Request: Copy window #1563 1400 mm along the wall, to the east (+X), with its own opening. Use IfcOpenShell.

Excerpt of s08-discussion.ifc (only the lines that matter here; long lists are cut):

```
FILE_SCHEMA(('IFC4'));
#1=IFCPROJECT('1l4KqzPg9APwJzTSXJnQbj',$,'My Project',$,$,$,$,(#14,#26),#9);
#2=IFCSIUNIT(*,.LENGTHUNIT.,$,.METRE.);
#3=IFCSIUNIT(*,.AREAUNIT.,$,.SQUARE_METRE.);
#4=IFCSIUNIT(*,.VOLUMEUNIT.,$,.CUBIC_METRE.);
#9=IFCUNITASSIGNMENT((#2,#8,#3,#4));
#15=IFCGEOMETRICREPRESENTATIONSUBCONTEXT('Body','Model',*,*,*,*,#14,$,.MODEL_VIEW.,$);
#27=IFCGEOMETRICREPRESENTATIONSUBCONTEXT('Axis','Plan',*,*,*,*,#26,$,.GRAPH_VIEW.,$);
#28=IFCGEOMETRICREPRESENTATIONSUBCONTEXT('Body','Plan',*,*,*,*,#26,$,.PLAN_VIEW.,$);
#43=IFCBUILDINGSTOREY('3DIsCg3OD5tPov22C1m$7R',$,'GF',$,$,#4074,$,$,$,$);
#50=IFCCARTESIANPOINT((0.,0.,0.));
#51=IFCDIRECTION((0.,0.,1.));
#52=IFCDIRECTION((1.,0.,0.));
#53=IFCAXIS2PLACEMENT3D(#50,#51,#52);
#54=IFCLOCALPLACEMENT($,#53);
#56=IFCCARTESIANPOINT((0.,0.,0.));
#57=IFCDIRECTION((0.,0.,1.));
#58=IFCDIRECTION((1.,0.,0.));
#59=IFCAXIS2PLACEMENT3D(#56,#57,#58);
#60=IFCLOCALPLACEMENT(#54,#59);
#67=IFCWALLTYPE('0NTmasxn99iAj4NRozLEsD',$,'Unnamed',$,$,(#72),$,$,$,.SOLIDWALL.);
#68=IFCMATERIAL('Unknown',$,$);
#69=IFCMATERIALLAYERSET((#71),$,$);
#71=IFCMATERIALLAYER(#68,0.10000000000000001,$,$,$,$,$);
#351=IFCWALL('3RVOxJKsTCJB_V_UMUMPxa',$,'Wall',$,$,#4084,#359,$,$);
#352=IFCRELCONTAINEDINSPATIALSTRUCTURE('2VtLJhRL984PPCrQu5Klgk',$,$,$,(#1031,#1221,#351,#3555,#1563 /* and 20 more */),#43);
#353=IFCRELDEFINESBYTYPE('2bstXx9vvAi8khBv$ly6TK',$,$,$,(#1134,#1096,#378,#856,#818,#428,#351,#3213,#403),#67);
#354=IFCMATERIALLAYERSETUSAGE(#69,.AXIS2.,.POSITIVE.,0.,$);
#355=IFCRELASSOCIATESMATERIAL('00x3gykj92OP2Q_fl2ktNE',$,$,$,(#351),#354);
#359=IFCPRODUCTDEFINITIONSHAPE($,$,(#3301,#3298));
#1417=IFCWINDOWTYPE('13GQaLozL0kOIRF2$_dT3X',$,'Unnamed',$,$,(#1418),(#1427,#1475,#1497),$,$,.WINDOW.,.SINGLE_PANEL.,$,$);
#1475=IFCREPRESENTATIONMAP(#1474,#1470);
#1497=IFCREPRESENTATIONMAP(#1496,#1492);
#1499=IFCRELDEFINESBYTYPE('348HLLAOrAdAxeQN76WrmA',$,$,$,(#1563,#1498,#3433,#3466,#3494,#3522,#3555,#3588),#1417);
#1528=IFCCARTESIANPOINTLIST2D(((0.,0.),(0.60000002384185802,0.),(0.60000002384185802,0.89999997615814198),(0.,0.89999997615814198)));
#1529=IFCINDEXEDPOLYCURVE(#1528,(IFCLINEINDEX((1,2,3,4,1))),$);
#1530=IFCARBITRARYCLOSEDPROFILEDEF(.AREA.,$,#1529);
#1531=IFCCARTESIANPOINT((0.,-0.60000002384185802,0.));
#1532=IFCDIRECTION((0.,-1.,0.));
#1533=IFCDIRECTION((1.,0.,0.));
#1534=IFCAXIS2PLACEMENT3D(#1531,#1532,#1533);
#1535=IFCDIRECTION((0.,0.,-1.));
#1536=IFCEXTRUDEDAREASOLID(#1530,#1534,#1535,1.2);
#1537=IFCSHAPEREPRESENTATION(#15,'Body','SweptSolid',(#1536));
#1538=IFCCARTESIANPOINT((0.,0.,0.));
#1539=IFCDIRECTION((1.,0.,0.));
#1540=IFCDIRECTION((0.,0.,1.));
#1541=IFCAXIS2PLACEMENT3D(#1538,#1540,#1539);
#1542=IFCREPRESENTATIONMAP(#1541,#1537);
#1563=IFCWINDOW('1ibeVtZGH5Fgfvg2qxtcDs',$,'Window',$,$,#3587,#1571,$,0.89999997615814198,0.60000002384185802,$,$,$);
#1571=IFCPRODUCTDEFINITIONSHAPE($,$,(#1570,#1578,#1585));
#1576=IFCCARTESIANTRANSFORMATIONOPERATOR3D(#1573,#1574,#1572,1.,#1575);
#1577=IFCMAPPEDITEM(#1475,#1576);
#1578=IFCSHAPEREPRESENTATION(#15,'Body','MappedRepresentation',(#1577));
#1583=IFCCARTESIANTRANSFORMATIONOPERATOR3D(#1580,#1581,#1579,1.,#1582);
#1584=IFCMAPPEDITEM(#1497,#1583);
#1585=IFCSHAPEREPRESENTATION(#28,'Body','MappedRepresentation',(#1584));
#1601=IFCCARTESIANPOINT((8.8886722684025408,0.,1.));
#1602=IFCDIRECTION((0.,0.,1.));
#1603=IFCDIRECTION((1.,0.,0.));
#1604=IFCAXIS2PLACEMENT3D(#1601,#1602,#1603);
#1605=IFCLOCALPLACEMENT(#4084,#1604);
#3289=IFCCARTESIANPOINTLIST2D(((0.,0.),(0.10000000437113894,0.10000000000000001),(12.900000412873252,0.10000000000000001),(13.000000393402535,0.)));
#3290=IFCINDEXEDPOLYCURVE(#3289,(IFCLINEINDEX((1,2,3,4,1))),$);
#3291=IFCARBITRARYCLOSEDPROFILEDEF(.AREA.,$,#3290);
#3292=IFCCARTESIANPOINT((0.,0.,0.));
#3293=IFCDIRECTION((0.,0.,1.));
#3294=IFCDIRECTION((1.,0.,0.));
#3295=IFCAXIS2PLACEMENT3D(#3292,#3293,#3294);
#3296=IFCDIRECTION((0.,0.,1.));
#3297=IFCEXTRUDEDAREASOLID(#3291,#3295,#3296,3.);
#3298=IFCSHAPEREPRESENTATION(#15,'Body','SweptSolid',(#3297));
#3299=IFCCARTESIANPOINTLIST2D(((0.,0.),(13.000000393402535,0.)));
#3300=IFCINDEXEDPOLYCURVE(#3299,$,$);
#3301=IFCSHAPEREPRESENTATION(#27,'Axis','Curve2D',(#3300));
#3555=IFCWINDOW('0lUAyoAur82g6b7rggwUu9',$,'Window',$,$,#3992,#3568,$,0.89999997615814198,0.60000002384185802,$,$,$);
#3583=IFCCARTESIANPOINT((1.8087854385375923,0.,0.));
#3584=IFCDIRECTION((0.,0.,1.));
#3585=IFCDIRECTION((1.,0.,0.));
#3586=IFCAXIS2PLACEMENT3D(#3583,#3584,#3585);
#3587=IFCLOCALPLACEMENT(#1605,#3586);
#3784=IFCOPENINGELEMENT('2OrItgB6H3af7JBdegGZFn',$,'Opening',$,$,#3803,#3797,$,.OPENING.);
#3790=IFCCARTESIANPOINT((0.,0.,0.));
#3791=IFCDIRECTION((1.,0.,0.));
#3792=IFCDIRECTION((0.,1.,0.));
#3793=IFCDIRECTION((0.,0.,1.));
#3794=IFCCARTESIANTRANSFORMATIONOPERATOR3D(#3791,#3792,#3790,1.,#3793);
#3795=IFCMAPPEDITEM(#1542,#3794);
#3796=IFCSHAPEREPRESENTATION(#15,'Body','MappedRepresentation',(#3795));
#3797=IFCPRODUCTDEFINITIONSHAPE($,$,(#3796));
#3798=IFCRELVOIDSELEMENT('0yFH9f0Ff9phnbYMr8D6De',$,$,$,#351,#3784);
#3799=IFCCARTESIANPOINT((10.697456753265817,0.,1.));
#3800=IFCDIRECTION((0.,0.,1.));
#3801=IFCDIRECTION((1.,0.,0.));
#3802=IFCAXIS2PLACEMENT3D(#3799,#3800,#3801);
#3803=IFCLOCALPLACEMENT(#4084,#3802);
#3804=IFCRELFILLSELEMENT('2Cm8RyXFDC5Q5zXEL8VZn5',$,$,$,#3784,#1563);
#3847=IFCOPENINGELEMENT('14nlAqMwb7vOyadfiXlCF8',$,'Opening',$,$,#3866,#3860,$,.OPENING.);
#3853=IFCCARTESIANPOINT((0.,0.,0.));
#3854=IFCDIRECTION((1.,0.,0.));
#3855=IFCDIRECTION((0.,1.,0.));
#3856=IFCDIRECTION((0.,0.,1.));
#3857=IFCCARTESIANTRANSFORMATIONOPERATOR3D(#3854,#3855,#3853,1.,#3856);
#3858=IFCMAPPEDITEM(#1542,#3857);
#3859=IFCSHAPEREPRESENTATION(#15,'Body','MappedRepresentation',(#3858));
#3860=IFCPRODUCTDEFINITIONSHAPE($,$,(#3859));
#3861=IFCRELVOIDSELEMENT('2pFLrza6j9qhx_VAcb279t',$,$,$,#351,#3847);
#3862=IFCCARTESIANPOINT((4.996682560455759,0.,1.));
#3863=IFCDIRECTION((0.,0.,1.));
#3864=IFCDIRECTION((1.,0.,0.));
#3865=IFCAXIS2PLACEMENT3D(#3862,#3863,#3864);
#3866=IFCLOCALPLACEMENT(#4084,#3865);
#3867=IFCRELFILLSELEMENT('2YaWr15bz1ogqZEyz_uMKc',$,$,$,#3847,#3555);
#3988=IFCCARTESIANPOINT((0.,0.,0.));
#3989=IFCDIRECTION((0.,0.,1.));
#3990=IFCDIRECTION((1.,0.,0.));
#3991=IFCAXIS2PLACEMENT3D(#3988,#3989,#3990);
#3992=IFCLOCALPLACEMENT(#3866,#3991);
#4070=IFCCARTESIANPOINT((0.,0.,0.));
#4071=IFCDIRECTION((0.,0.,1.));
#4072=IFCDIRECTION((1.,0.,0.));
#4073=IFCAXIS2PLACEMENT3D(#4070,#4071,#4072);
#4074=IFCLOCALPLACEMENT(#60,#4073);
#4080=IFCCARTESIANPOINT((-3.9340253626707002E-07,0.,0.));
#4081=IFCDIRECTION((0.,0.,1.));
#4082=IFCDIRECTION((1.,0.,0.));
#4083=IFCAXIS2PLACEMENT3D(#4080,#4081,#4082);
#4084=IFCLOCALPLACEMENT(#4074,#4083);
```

```python
import ifcopenshell
import ifcopenshell.api.feature
import ifcopenshell.api.geometry
import ifcopenshell.api.root
import ifcopenshell.geom
import ifcopenshell.util.element
import ifcopenshell.util.placement
import ifcopenshell.util.shape

model = ifcopenshell.open("s08-discussion.ifc")
settings = ifcopenshell.geom.settings()


def volume(element):
    """Net volume in cubic metres, openings subtracted."""
    shape = ifcopenshell.geom.create_shape(settings, element)
    return ifcopenshell.util.shape.get_volume(shape.geometry)


window = model.by_guid("1ibeVtZGH5Fgfvg2qxtcDs")
opening = window.FillsVoids[0].RelatingOpeningElement
wall = opening.VoidsElements[0].RelatingBuildingElement
before = volume(wall)
shift = ifcopenshell.util.placement.get_local_placement(wall.ObjectPlacement)[:3, 0] * 1.4

# copy_class copies the void relationship, type, container and properties, but no geometry.
new_opening = ifcopenshell.api.root.copy_class(model, product=opening)
new_opening.Representation = ifcopenshell.util.element.copy_deep(
    model, opening.Representation, exclude=["IfcGeometricRepresentationContext", "IfcRepresentationMap"]
)
new_window = ifcopenshell.api.root.copy_class(model, product=window)
new_window.Representation = ifcopenshell.util.element.copy_deep(
    model, window.Representation, exclude=["IfcGeometricRepresentationContext", "IfcRepresentationMap"]
)
ifcopenshell.api.feature.add_filling(model, opening=new_opening, element=new_window)

for old, new in ((opening, new_opening), (window, new_window)):
    matrix = ifcopenshell.util.placement.get_local_placement(old.ObjectPlacement)
    matrix[:3, 3] += shift
    ifcopenshell.api.geometry.edit_object_placement(model, product=new, matrix=matrix, is_si=False)

after = volume(wall)

print(f"wall volume {before:.3f} -> {after:.3f} m3")

model.write("s08-discussion_rev.ifc")
```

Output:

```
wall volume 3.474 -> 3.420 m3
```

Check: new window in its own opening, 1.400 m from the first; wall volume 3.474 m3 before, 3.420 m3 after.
